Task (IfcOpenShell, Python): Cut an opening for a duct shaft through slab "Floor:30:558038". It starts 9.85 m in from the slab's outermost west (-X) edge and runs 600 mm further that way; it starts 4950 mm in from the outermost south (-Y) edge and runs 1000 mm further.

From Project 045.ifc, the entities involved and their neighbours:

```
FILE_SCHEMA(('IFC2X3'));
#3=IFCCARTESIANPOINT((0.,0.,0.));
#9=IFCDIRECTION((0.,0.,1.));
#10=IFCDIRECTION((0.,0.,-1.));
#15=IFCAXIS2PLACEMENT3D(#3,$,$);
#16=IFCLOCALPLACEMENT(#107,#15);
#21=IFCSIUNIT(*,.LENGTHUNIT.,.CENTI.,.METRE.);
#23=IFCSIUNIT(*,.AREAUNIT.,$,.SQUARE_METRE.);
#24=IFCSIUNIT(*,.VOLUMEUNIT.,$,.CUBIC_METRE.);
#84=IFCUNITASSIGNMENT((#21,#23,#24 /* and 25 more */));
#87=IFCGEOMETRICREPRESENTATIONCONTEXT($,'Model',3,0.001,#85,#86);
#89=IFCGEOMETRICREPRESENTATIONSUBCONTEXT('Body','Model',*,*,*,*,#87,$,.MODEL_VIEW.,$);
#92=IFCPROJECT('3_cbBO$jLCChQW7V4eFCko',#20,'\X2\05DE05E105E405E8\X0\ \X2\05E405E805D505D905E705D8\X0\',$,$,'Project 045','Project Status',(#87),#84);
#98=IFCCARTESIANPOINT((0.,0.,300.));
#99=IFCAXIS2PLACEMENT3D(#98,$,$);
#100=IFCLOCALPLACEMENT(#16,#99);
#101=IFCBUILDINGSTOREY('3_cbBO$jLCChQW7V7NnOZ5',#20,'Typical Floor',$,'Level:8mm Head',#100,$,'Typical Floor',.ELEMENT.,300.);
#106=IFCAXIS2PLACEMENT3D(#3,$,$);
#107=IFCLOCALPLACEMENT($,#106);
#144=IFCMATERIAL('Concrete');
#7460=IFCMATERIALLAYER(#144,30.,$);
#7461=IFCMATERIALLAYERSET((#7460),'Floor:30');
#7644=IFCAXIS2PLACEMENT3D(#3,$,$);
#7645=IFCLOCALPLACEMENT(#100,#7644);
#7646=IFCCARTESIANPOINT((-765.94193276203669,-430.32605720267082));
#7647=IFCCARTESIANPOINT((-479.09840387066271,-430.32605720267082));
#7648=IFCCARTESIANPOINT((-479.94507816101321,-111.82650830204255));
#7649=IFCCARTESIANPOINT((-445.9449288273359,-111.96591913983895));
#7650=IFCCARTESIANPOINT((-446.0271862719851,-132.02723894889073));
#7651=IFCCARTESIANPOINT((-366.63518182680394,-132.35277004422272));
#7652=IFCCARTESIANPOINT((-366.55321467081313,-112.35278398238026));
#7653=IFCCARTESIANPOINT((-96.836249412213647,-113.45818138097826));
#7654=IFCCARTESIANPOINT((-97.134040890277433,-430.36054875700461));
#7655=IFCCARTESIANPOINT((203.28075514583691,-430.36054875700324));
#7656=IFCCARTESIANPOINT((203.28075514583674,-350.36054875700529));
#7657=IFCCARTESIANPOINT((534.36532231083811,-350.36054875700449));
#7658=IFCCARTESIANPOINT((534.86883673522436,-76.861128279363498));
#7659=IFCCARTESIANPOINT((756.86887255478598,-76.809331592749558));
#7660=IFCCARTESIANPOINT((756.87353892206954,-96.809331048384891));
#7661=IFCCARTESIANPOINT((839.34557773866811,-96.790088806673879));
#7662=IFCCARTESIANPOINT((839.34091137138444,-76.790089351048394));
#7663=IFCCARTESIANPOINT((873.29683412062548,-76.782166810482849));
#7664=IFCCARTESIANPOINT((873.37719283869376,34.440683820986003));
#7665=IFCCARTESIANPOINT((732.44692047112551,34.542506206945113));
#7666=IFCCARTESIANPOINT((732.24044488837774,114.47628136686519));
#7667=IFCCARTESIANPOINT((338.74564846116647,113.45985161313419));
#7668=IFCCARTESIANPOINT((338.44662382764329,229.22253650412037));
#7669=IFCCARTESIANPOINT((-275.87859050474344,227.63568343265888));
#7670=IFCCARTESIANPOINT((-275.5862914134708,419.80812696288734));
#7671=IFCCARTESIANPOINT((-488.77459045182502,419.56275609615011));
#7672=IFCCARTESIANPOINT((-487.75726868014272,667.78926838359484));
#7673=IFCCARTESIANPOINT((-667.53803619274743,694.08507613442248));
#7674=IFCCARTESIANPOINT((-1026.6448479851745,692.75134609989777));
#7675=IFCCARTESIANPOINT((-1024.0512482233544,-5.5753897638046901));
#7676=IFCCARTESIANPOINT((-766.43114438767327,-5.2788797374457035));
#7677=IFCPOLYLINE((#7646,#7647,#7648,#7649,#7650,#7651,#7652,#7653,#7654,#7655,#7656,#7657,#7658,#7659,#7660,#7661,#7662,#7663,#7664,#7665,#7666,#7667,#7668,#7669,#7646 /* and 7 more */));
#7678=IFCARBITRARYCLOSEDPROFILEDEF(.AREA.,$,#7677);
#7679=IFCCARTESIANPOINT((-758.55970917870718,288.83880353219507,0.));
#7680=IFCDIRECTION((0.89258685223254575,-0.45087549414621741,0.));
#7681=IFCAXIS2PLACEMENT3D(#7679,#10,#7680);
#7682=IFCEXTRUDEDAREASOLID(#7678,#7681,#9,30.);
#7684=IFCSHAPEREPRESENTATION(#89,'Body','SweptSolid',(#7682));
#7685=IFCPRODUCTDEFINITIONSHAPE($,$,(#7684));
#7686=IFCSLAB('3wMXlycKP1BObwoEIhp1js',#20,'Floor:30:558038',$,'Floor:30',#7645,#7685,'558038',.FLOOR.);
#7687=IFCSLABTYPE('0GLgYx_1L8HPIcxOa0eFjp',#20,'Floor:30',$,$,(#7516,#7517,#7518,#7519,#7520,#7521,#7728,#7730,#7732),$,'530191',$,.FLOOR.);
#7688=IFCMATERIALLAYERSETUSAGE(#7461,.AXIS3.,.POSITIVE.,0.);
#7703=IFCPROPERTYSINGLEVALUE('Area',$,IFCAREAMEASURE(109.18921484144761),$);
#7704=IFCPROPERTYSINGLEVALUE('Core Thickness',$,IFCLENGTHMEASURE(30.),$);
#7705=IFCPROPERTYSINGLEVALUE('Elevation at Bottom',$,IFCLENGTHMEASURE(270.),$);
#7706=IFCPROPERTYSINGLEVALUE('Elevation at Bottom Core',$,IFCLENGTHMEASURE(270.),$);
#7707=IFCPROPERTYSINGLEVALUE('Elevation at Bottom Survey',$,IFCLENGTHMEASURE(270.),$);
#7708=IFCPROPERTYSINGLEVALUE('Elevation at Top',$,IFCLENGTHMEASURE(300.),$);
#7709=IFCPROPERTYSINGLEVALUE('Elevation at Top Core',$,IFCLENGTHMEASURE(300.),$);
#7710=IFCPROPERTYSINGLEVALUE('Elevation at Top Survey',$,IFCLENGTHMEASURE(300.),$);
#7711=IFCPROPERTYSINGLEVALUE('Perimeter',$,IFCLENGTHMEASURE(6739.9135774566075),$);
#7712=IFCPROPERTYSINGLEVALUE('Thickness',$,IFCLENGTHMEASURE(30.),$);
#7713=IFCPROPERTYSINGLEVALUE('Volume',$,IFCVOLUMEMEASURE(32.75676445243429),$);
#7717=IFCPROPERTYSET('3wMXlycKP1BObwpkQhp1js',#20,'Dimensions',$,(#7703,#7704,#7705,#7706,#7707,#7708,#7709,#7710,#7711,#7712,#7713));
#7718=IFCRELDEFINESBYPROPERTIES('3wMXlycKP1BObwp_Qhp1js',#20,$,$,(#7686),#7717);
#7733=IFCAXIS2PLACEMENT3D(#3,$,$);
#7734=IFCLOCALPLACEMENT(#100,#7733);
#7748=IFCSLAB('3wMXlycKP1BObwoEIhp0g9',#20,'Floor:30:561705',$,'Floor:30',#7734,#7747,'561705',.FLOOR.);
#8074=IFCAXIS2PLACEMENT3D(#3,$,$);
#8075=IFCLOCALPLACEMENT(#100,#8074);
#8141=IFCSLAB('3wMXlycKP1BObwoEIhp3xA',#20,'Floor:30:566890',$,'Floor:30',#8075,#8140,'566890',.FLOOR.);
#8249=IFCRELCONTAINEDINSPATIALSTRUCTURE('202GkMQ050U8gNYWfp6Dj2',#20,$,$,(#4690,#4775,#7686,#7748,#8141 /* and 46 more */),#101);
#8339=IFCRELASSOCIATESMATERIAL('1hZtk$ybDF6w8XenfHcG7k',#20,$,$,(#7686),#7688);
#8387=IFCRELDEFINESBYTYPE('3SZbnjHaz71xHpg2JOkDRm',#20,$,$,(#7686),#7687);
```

```python
import numpy as np
import ifcopenshell
import ifcopenshell.api.feature
import ifcopenshell.api.geometry
import ifcopenshell.api.pset
import ifcopenshell.api.root
import ifcopenshell.geom
import ifcopenshell.util.element
import ifcopenshell.util.placement
import ifcopenshell.util.representation
import ifcopenshell.util.shape
import ifcopenshell.util.unit

model = ifcopenshell.open("Project 045.ifc")
unit_scale = ifcopenshell.util.unit.calculate_unit_scale(model)
area_scale = ifcopenshell.util.unit.calculate_unit_scale(model, "AREAUNIT")
volume_scale = ifcopenshell.util.unit.calculate_unit_scale(model, "VOLUMEUNIT")
settings = ifcopenshell.geom.settings()


def volume(element):
    """Net volume in cubic metres, openings subtracted."""
    shape = ifcopenshell.geom.create_shape(settings, element)
    return ifcopenshell.util.shape.get_volume(shape.geometry)


slab = model.by_guid("3wMXlycKP1BObwoEIhp1js")
before = volume(slab)

# Extent in the slab's own axes, in metres. The edges named are its -X and -Y sides.
slab_shape = ifcopenshell.geom.create_shape(settings, slab)
vertices = ifcopenshell.util.shape.get_vertices(slab_shape.geometry)
x_min, y_min, bottom = vertices.min(axis=0)
top = vertices[:, 2].max()

opening = ifcopenshell.api.root.create_entity(model, ifc_class="IfcOpeningElement", name="Duct shaft opening")
context = ifcopenshell.util.representation.get_context(model, "Model", "Body", "MODEL_VIEW")
width, depth = 0.6, 1
outline = [(0.0, 0.0), (width, 0.0), (width, depth), (0.0, depth), (0.0, 0.0)]
# Overshoot both faces by 50 mm so the cut is clean.
shape = ifcopenshell.api.geometry.add_slab_representation(
    model, context=context, depth=top - bottom + 0.1, polyline=outline
)
ifcopenshell.api.geometry.assign_representation(model, product=opening, representation=shape)

matrix = ifcopenshell.util.placement.get_local_placement(slab.ObjectPlacement)
matrix[:, 3] = matrix @ np.append(np.array([x_min + 9.85, y_min + 4.95, bottom - 0.05]) / unit_scale, 1.0)
ifcopenshell.api.geometry.edit_object_placement(model, product=opening, matrix=matrix, is_si=False)
ifcopenshell.api.feature.add_feature(model, feature=opening, element=slab)

after = volume(slab)

# Update the slab's stored quantities.
pset = model.by_id(ifcopenshell.util.element.get_pset(slab, "Dimensions", should_inherit=False)["id"])
ifcopenshell.api.pset.edit_pset(model, pset=pset, properties={
    "Area": model.create_entity("IfcAreaMeasure", after / (top - bottom) / area_scale),
    "Volume": model.create_entity("IfcVolumeMeasure", after / volume_scale),
})

print(f"slab volume {before:.3f} -> {after:.3f} m3")

model.write("Project 045_updated.ifc")
```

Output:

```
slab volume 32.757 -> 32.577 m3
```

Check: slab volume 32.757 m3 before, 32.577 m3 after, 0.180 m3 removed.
